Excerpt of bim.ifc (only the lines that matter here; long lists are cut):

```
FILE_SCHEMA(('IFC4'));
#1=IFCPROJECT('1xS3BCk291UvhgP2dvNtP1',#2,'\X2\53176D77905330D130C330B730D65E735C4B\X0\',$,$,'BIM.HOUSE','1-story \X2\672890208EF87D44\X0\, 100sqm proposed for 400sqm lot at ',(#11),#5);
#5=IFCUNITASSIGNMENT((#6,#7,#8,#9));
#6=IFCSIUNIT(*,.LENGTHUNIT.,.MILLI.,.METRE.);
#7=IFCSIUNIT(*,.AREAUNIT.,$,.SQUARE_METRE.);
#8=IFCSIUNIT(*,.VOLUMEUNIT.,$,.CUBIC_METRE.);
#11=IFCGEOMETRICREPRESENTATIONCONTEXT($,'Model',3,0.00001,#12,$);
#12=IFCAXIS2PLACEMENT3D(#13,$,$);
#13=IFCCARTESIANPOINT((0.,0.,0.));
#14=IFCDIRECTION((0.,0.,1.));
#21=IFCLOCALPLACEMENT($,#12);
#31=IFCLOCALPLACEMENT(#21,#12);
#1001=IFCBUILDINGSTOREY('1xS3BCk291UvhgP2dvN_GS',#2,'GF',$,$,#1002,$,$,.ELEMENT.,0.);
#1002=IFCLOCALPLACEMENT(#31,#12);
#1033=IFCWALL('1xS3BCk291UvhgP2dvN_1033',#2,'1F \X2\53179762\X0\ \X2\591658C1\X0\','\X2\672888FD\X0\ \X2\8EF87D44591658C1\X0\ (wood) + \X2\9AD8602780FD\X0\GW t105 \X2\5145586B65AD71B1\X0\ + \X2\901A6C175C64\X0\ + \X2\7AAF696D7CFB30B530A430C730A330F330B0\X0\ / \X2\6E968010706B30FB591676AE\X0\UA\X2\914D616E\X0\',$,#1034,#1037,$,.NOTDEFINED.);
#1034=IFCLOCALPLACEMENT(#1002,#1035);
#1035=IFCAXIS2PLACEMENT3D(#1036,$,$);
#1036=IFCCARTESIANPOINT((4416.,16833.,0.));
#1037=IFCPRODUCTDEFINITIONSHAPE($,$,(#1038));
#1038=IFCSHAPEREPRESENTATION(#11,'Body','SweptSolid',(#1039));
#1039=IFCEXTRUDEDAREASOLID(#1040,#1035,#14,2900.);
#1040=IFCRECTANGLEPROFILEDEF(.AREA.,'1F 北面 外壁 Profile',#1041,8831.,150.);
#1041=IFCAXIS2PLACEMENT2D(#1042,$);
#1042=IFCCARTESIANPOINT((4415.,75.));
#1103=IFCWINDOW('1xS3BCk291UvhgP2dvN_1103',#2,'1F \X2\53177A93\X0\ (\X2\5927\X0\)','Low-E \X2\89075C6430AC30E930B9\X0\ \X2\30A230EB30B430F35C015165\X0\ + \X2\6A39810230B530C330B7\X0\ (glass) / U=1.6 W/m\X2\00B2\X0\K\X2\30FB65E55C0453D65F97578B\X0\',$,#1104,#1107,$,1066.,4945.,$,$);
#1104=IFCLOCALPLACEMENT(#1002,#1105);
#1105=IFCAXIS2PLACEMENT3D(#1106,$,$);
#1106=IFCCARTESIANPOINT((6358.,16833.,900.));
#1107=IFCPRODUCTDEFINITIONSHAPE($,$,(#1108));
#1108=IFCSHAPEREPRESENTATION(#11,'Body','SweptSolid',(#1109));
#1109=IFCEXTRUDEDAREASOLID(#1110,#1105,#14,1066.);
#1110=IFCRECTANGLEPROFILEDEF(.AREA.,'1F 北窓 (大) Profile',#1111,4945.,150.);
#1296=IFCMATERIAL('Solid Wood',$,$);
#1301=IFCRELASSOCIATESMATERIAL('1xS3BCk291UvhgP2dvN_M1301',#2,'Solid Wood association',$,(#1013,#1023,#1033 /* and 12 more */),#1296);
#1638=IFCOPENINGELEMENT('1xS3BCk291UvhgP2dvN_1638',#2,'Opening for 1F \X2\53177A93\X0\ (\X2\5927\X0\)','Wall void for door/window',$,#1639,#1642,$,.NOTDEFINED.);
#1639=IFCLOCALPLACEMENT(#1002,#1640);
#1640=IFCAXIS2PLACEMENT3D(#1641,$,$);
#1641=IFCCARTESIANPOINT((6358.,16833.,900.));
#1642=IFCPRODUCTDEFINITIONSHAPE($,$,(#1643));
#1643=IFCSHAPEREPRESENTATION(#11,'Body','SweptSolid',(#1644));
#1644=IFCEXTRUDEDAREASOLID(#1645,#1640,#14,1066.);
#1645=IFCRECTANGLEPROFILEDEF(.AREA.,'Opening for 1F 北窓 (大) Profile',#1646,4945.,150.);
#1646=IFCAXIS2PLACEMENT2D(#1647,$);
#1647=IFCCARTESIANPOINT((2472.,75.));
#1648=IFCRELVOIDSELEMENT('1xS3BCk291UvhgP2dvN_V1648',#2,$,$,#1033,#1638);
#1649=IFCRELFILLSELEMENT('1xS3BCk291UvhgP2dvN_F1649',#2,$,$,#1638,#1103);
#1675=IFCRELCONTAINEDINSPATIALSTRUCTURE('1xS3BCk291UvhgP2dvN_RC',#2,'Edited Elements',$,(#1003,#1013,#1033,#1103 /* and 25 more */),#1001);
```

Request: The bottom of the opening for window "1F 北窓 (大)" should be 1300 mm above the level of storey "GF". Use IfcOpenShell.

```python
import numpy as np
import ifcopenshell
import ifcopenshell.api.geometry
import ifcopenshell.geom
import ifcopenshell.util.element
import ifcopenshell.util.placement
import ifcopenshell.util.shape
import ifcopenshell.util.unit

model = ifcopenshell.open("bim.ifc")
unit_scale = ifcopenshell.util.unit.calculate_unit_scale(model)

window = model.by_guid("1xS3BCk291UvhgP2dvN_1103")
opening = window.FillsVoids[0].RelatingOpeningElement
storey = ifcopenshell.util.element.get_container(window, ifc_class="IfcBuildingStorey")
level = ifcopenshell.util.placement.get_local_placement(storey.ObjectPlacement)[2, 3]

# The opening's origin need not be at the sill, so measure its lowest point.
shape = ifcopenshell.geom.create_shape(ifcopenshell.geom.settings(), opening)
bottom = ifcopenshell.util.shape.get_shape_bottom_elevation(shape, shape.geometry) / unit_scale
dz = level + 1.3 / unit_scale - bottom

shift = np.array([0.0, 0.0, dz])
# The window is not placed relative to its opening, so move both.
for product in (opening, window):
    matrix = ifcopenshell.util.placement.get_local_placement(product.ObjectPlacement)
    matrix[:3, 3] += shift
    ifcopenshell.api.geometry.edit_object_placement(model, product=product, matrix=matrix, is_si=False)

print(f"moved by {dz * unit_scale:+.3f} m")

model.write("bim_rev.ifc")
```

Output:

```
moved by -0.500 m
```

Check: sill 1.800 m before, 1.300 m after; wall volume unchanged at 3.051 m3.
